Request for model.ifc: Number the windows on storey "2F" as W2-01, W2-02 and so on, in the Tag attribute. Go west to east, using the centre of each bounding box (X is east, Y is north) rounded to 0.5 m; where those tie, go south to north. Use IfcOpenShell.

First a look at what the model holds.

```python
import ifcopenshell
import ifcopenshell.util.element
import ifcopenshell.util.placement

model = ifcopenshell.open("model.ifc")
print(model.schema)
storey = next(s for s in model.by_type("IfcBuildingStorey") if s.Name == "2F")
windows = [e for e in ifcopenshell.util.element.get_decomposition(storey) if e.is_a("IfcWindow")]
for e in sorted(windows, key=lambda e: e.id()):
    origin = ifcopenshell.util.placement.get_local_placement(e.ObjectPlacement)[:3, 3]
    print(e.id(), e.Tag, e.Name, origin.round(2) + 0.0, sep=" | ")
```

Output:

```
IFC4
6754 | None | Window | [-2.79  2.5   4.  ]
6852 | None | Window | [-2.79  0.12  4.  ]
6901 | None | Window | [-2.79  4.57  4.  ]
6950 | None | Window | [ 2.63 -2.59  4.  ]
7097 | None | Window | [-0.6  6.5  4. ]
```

```python
import ifcopenshell
import ifcopenshell.geom
import ifcopenshell.util.element
import ifcopenshell.util.shape

model = ifcopenshell.open("model.ifc")
settings = ifcopenshell.geom.settings()
settings.set("use-world-coords", True)


def centre(element):
    shape = ifcopenshell.geom.create_shape(settings, element)
    return ifcopenshell.util.shape.get_bbox_centroid(shape.geometry)


storey = next(s for s in model.by_type("IfcBuildingStorey") if s.Name == "2F")
windows = [e for e in ifcopenshell.util.element.get_decomposition(storey) if e.is_a("IfcWindow")]

# Insertion points can sit at a corner or the storey origin, so sort by the geometry (in metres).
centres = {e: centre(e) for e in windows}
windows.sort(key=lambda e: (round(centres[e][0] / 0.5), centres[e][1]))

for i, e in enumerate(windows, start=1):
    number = f"W2-{i:02d}"
    e.Tag = number
    print(e.id(), number)

model.write("model_rev.ifc")
```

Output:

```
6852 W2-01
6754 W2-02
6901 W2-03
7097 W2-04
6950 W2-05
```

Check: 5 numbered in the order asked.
